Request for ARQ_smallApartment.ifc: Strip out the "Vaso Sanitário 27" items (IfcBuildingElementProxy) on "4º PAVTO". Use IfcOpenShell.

First a look at what the model holds.

```python
import ifcopenshell
import ifcopenshell.util.element

model = ifcopenshell.open("ARQ_smallApartment.ifc")
print(model.schema)
storey = next(s for s in model.by_type("IfcBuildingStorey") if s.Name == "4º PAVTO")
proxies = [e for e in ifcopenshell.util.element.get_decomposition(storey) if e.is_a("IfcBuildingElementProxy")]
seen = {}
for e in proxies:
    element_type = ifcopenshell.util.element.get_type(e)
    name = element_type.Name if element_type not in (None, e) else None
    seen[name] = seen.get(name, 0) + 1
for name, count in sorted(seen.items(), key=str):
    print(count, "x", name)
```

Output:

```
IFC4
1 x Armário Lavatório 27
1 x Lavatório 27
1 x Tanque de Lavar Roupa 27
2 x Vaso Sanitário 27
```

```python
import ifcopenshell
import ifcopenshell.api.root
import ifcopenshell.util.element

model = ifcopenshell.open("ARQ_smallApartment.ifc")

storey = next(s for s in model.by_type("IfcBuildingStorey") if s.Name == "4º PAVTO")
proxies = [e for e in ifcopenshell.util.element.get_decomposition(storey) if e.is_a("IfcBuildingElementProxy")]
targets = [e for e in proxies if (t := ifcopenshell.util.element.get_type(e)) not in (None, e) and t.Name == "Vaso Sanitário 27"]

for e in targets:
    ifcopenshell.api.root.remove_product(model, product=e)
print(len(targets), "removed")

model.write("ARQ_smallApartment_edited.ifc")
```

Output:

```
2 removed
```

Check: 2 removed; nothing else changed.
